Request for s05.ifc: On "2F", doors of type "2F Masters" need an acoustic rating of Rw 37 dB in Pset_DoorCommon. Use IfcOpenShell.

First a look at what the model holds.

```python
import ifcopenshell
import ifcopenshell.util.element

model = ifcopenshell.open("s05.ifc")
print(model.schema)
storey = next(s for s in model.by_type("IfcBuildingStorey") if s.Name == "2F")
doors = [e for e in ifcopenshell.util.element.get_decomposition(storey) if e.is_a("IfcDoor")]
seen = {}
for e in doors:
    element_type = ifcopenshell.util.element.get_type(e)
    key = (element_type.Name if element_type != e and element_type else None, ifcopenshell.util.element.get_pset(e, "Pset_DoorCommon", "AcousticRating"))
    seen[key] = seen.get(key, 0) + 1
for (name, value), count in sorted(seen.items(), key=str):
    print(count, "x", name, "|", value)
```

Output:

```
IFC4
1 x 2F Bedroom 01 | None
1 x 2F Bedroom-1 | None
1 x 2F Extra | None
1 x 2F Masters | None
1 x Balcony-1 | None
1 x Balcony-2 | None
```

```python
import ifcopenshell
import ifcopenshell.api.pset
import ifcopenshell.util.element

model = ifcopenshell.open("s05.ifc")

storey = next(s for s in model.by_type("IfcBuildingStorey") if s.Name == "2F")
doors = [e for e in ifcopenshell.util.element.get_decomposition(storey) if e.is_a("IfcDoor")]

count = 0
for e in doors:
    element_type = ifcopenshell.util.element.get_type(e)
    if element_type in (None, e) or element_type.Name != "2F Masters":
        continue
    # add_pset returns the element's existing set when there is one.
    pset = ifcopenshell.api.pset.add_pset(model, product=e, name="Pset_DoorCommon")
    ifcopenshell.api.pset.edit_pset(model, pset=pset, properties={"AcousticRating": "Rw 37 dB"})
    count += 1

print(count, "doors updated")

model.write("s05_rev.ifc")
```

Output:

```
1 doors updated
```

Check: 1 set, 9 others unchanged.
